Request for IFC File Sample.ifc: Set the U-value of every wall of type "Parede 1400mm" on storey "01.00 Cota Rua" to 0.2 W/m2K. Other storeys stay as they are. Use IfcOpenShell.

First a look at what the model holds.

```python
import ifcopenshell
import ifcopenshell.util.element

model = ifcopenshell.open("IFC File Sample.ifc")
print(model.schema)
storey = next(s for s in model.by_type("IfcBuildingStorey") if s.Name == "01.00 Cota Rua")
walls = [e for e in ifcopenshell.util.element.get_decomposition(storey) if e.is_a("IfcWall")]
seen = {}
for e in walls:
    element_type = ifcopenshell.util.element.get_type(e)
    key = (element_type.Name if element_type != e and element_type else None, ifcopenshell.util.element.get_pset(e, "Pset_WallCommon", "ThermalTransmittance"))
    seen[key] = seen.get(key, 0) + 1
for (name, value), count in sorted(seen.items(), key=str):
    print(count, "x", name, "|", value)
```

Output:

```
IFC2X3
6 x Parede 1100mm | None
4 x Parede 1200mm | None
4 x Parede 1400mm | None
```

```python
import ifcopenshell
import ifcopenshell.api.pset
import ifcopenshell.util.element

model = ifcopenshell.open("IFC File Sample.ifc")

storey = next(s for s in model.by_type("IfcBuildingStorey") if s.Name == "01.00 Cota Rua")
walls = [e for e in ifcopenshell.util.element.get_decomposition(storey) if e.is_a("IfcWall")]

count = 0
for e in walls:
    element_type = ifcopenshell.util.element.get_type(e)
    if element_type in (None, e) or element_type.Name != "Parede 1400mm":
        continue
    # add_pset returns the element's existing set when there is one.
    pset = ifcopenshell.api.pset.add_pset(model, product=e, name="Pset_WallCommon")
    ifcopenshell.api.pset.edit_pset(model, pset=pset, properties={"ThermalTransmittance": 0.2})
    count += 1

print(count, "walls updated")

model.write("IFC File Sample_updated.ifc")
```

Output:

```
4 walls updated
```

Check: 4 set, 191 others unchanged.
